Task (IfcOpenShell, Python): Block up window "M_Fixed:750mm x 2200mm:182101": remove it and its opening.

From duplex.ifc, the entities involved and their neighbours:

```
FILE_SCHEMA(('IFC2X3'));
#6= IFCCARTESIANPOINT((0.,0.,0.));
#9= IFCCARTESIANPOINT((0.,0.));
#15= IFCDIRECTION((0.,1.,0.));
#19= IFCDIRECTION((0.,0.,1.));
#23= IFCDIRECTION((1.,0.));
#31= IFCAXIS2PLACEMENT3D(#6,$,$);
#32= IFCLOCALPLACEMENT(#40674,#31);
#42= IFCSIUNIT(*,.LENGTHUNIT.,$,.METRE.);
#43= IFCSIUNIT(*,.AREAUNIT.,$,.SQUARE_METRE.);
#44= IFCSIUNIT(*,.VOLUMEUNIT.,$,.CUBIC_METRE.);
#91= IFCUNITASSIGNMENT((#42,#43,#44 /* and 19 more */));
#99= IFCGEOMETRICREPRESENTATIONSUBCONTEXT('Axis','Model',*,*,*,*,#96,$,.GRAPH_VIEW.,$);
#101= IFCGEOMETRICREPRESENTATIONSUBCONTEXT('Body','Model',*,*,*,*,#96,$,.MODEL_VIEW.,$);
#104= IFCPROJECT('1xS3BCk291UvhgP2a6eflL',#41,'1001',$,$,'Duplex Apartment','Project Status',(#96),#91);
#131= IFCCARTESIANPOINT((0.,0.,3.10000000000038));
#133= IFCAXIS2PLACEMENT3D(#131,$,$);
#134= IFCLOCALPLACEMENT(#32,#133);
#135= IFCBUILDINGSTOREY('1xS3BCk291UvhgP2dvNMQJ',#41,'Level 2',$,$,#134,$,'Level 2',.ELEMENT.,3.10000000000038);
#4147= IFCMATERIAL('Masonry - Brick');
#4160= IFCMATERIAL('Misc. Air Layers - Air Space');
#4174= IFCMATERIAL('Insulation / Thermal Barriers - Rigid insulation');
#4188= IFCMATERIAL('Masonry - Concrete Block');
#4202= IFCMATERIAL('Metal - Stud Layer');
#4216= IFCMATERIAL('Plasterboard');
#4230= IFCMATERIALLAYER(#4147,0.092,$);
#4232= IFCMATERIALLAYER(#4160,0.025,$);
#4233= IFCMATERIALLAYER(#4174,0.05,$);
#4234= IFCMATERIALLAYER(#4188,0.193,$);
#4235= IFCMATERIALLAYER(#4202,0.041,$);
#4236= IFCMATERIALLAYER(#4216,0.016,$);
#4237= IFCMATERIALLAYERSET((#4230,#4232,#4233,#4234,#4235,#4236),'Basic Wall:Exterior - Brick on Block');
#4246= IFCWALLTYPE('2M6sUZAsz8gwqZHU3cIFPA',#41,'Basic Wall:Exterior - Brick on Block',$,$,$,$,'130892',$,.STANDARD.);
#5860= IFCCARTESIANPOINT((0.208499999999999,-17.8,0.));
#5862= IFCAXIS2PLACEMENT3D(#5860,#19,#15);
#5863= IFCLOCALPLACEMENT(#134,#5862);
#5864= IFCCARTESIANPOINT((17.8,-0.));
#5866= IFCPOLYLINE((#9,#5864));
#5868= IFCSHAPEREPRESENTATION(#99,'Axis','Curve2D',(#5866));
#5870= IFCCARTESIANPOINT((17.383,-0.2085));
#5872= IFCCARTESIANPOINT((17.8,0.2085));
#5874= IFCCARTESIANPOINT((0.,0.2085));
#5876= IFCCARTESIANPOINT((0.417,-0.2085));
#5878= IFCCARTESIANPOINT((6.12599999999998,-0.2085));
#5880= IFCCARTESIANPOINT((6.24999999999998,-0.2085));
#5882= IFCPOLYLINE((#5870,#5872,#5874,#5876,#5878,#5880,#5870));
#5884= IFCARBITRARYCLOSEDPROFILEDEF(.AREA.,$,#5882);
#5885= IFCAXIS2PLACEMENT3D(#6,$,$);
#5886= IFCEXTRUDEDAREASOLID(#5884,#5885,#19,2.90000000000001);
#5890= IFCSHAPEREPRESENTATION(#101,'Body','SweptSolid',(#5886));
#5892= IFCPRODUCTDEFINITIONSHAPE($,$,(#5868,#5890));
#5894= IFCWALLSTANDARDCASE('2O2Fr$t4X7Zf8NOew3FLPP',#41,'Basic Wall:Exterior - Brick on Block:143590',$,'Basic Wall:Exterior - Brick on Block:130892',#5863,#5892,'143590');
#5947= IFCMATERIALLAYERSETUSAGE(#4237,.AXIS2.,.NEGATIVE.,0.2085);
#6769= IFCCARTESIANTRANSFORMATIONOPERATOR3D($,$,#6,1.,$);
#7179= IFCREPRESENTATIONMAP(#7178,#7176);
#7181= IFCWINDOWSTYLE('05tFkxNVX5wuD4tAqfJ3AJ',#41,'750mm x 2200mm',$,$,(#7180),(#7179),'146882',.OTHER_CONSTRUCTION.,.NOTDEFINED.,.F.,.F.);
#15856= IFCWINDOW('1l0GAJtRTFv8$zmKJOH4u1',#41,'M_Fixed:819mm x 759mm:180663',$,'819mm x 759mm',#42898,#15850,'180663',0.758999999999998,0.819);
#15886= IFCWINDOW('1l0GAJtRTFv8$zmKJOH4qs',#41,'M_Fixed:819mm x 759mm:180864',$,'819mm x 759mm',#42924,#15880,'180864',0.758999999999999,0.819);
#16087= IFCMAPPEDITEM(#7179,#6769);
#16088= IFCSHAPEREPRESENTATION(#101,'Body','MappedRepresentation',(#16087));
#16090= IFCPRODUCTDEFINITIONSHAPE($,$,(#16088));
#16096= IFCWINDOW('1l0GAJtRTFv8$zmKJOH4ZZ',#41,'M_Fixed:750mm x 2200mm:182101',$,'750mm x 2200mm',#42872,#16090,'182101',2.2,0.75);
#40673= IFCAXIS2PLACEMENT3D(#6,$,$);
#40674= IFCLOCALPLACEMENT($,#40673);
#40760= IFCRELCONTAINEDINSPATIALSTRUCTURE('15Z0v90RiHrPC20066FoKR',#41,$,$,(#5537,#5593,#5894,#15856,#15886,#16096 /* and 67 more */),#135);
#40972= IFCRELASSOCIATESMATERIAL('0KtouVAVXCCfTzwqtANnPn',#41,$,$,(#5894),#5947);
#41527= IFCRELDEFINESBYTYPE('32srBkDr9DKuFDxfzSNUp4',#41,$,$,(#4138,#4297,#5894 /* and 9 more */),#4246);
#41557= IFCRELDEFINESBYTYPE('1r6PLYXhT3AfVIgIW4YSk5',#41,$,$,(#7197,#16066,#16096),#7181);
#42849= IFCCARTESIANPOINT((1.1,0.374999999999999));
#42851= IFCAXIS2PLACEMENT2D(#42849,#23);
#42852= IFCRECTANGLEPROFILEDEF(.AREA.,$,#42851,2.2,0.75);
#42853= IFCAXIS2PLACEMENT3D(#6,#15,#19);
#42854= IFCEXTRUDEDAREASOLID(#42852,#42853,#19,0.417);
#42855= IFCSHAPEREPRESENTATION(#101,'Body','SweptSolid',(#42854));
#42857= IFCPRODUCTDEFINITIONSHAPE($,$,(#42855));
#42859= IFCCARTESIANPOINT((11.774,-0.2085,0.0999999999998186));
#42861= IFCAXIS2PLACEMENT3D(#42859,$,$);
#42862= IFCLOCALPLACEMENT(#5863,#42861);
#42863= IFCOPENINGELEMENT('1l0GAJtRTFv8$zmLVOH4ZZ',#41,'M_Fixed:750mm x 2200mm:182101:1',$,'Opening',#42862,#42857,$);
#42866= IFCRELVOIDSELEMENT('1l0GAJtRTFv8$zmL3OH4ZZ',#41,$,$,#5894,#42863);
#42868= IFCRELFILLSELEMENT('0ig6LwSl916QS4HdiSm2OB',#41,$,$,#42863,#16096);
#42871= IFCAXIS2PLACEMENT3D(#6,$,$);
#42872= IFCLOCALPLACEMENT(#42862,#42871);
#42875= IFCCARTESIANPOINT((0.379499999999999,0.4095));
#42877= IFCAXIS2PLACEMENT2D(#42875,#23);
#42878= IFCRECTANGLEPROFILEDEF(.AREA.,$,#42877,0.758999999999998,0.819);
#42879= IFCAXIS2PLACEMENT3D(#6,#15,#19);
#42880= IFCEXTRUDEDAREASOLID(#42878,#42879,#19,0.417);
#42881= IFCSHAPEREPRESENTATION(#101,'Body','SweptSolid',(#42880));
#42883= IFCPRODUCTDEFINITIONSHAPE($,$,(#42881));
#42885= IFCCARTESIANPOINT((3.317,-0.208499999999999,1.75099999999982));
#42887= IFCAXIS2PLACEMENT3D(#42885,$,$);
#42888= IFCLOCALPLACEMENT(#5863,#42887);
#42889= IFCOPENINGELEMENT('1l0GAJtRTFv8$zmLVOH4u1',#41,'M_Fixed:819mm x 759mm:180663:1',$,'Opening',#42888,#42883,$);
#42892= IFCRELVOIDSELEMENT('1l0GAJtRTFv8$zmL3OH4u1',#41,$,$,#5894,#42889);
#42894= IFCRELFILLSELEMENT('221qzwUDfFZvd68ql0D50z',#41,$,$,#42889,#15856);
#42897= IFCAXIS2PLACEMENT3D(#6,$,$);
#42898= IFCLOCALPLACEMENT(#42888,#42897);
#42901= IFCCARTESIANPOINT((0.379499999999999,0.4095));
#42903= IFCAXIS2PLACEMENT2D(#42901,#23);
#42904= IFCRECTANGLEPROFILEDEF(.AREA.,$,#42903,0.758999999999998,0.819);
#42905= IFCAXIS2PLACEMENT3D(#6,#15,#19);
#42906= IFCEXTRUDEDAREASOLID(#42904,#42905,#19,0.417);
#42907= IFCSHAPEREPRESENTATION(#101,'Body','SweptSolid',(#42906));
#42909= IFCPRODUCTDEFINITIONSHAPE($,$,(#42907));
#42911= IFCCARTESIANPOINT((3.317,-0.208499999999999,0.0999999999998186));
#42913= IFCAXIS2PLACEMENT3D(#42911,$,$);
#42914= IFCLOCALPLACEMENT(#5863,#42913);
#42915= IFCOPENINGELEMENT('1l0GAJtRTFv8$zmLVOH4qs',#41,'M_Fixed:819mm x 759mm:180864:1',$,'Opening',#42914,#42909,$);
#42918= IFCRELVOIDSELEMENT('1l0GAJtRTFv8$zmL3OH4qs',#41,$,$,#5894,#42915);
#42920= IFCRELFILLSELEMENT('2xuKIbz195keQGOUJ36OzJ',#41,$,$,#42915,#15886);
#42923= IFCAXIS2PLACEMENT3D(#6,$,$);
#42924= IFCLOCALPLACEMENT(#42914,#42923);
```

```python
import ifcopenshell
import ifcopenshell.api.feature
import ifcopenshell.api.root
import ifcopenshell.geom
import ifcopenshell.util.shape

model = ifcopenshell.open("duplex.ifc")
settings = ifcopenshell.geom.settings()


def volume(element):
    """Net volume in cubic metres, openings subtracted."""
    shape = ifcopenshell.geom.create_shape(settings, element)
    return ifcopenshell.util.shape.get_volume(shape.geometry)


window = model.by_guid("1l0GAJtRTFv8$zmKJOH4ZZ")
opening = window.FillsVoids[0].RelatingOpeningElement
wall = opening.VoidsElements[0].RelatingBuildingElement
before = volume(wall)

ifcopenshell.api.root.remove_product(model, product=window)
ifcopenshell.api.feature.remove_feature(model, feature=opening)

after = volume(wall)

print(f"wall volume {before:.3f} -> {after:.3f} m3")

model.write("duplex_updated.ifc")
```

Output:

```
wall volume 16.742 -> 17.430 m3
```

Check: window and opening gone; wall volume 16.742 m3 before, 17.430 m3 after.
